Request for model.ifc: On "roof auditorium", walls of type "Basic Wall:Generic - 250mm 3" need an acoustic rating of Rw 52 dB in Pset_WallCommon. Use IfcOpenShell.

First a look at what the model holds.

```python
import ifcopenshell
import ifcopenshell.util.element

model = ifcopenshell.open("model.ifc")
print(model.schema)
storey = next(s for s in model.by_type("IfcBuildingStorey") if s.Name == "roof auditorium")
walls = [e for e in ifcopenshell.util.element.get_decomposition(storey) if e.is_a("IfcWall")]
seen = {}
for e in walls:
    element_type = ifcopenshell.util.element.get_type(e)
    key = (element_type.Name if element_type != e and element_type else None, ifcopenshell.util.element.get_pset(e, "Pset_WallCommon", "AcousticRating"))
    seen[key] = seen.get(key, 0) + 1
for (name, value), count in sorted(seen.items(), key=str):
    print(count, "x", name, "|", value)
```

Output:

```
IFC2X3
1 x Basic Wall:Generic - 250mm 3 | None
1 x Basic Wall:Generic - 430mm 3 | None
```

```python
import ifcopenshell
import ifcopenshell.api.pset
import ifcopenshell.util.element

model = ifcopenshell.open("model.ifc")

storey = next(s for s in model.by_type("IfcBuildingStorey") if s.Name == "roof auditorium")
walls = [e for e in ifcopenshell.util.element.get_decomposition(storey) if e.is_a("IfcWall")]

count = 0
for e in walls:
    element_type = ifcopenshell.util.element.get_type(e)
    if element_type in (None, e) or element_type.Name != "Basic Wall:Generic - 250mm 3":
        continue
    # add_pset returns the element's existing set when there is one.
    pset = ifcopenshell.api.pset.add_pset(model, product=e, name="Pset_WallCommon")
    ifcopenshell.api.pset.edit_pset(model, pset=pset, properties={"AcousticRating": "Rw 52 dB"})
    count += 1

print(count, "walls updated")

model.write("model_v2.ifc")
```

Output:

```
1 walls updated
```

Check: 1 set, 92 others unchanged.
